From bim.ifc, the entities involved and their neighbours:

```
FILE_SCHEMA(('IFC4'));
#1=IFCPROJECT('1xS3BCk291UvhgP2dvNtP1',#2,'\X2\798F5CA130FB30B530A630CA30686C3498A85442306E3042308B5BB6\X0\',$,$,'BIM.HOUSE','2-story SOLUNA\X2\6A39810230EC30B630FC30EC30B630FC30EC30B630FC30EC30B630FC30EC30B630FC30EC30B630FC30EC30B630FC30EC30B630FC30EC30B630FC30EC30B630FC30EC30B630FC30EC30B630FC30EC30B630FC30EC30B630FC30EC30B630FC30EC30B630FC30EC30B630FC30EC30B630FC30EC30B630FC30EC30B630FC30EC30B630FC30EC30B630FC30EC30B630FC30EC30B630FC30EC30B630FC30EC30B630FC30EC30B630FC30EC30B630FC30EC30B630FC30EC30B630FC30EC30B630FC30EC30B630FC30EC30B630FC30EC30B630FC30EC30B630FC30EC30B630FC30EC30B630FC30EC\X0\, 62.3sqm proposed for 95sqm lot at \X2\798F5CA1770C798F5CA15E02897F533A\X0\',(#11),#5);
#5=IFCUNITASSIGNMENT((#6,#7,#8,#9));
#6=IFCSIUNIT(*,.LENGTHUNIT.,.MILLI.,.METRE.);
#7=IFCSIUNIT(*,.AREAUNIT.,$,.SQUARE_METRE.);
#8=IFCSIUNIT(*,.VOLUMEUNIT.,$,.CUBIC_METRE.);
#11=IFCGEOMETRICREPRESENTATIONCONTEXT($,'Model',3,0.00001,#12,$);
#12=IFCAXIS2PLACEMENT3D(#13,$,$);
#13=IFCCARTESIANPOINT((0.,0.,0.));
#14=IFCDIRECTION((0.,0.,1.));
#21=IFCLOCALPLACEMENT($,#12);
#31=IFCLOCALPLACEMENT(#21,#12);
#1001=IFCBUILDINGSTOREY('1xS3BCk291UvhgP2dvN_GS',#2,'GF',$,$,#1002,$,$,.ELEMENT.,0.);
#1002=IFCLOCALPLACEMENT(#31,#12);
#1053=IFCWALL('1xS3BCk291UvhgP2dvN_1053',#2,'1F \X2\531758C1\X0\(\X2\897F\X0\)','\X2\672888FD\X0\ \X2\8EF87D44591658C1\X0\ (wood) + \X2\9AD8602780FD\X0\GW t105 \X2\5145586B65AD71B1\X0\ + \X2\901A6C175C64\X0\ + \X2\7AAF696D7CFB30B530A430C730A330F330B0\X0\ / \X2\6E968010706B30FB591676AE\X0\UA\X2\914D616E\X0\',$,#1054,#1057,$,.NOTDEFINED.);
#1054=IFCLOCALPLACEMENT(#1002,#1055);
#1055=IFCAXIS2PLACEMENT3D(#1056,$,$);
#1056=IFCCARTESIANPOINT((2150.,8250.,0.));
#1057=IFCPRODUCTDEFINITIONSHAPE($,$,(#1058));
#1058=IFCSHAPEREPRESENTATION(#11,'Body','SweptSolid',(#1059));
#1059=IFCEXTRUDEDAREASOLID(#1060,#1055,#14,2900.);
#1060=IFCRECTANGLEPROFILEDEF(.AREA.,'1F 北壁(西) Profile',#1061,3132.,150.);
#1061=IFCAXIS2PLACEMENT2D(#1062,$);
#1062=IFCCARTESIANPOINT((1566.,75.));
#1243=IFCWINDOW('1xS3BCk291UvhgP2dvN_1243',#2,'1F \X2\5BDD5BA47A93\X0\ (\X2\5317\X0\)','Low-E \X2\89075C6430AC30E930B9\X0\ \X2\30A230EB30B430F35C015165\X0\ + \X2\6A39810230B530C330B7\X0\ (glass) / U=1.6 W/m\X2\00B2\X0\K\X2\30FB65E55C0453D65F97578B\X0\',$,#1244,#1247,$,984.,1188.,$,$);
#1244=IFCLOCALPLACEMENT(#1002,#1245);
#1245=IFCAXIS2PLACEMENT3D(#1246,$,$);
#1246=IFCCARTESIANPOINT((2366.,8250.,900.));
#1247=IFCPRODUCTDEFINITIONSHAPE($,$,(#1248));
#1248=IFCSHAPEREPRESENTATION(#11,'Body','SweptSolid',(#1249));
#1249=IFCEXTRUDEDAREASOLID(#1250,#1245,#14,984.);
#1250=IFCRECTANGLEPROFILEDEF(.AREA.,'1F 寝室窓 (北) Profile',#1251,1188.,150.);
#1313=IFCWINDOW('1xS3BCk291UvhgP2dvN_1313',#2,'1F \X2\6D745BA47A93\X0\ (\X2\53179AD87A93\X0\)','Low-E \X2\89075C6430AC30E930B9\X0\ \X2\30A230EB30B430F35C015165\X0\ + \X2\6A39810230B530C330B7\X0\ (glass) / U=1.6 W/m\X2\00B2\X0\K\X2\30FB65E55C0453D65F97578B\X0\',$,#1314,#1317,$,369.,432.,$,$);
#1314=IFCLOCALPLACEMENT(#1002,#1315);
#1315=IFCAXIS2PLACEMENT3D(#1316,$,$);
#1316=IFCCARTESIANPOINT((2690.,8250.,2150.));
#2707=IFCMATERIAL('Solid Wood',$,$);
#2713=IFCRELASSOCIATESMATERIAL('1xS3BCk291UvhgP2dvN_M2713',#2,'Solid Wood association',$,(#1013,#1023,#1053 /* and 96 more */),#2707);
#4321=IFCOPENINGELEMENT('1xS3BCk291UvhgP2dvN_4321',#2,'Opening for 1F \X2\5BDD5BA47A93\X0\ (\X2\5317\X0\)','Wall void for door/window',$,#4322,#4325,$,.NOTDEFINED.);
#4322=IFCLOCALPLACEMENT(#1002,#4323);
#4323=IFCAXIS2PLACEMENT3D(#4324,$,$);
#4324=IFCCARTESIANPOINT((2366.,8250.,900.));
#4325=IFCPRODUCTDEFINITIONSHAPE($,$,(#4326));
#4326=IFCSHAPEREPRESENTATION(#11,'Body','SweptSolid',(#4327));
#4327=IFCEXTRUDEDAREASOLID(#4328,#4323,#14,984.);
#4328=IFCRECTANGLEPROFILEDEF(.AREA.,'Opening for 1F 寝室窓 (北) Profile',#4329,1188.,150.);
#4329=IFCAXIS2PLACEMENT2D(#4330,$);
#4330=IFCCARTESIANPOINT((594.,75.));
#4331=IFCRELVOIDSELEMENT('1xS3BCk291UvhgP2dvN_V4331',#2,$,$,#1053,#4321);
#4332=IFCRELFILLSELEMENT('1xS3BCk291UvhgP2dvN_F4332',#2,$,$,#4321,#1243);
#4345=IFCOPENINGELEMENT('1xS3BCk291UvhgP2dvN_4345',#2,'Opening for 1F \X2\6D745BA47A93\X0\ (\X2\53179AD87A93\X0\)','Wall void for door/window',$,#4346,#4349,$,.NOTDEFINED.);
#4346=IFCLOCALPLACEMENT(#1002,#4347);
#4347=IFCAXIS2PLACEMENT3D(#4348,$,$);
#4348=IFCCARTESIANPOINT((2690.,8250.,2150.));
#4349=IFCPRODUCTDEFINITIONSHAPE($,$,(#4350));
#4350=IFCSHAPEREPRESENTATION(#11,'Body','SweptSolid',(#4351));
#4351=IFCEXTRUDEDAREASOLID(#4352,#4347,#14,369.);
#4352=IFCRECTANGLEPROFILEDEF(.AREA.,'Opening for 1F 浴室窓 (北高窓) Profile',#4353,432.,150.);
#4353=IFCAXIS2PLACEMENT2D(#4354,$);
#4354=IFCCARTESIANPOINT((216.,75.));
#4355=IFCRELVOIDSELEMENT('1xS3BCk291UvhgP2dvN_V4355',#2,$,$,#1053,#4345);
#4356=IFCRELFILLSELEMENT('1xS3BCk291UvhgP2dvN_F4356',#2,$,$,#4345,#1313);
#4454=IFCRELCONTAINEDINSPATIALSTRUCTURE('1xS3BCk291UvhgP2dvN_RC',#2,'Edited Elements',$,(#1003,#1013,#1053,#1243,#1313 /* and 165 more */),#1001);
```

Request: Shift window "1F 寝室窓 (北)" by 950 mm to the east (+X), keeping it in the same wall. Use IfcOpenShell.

```python
import ifcopenshell
import ifcopenshell.api.geometry
import ifcopenshell.util.placement
import ifcopenshell.util.unit

model = ifcopenshell.open("bim.ifc")
unit_scale = ifcopenshell.util.unit.calculate_unit_scale(model)

window = model.by_id(1243)
opening = window.FillsVoids[0].RelatingOpeningElement
wall = opening.VoidsElements[0].RelatingBuildingElement

wall_matrix = ifcopenshell.util.placement.get_local_placement(wall.ObjectPlacement)
shift = wall_matrix[:3, 0] * 0.95 / unit_scale
before = ifcopenshell.util.placement.get_local_placement(window.ObjectPlacement)[:3, 3].copy()

# The window is not placed relative to its opening, so move both.
for product in (opening, window):
    matrix = ifcopenshell.util.placement.get_local_placement(product.ObjectPlacement)
    matrix[:3, 3] += shift
    ifcopenshell.api.geometry.edit_object_placement(model, product=product, matrix=matrix, is_si=False)

after = ifcopenshell.util.placement.get_local_placement(window.ObjectPlacement)[:3, 3]
print("window moved by", (after - before).round(3) + 0.0)

model.write("bim_rev.ifc")
```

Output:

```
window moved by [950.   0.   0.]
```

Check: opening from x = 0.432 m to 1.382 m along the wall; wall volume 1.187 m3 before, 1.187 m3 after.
